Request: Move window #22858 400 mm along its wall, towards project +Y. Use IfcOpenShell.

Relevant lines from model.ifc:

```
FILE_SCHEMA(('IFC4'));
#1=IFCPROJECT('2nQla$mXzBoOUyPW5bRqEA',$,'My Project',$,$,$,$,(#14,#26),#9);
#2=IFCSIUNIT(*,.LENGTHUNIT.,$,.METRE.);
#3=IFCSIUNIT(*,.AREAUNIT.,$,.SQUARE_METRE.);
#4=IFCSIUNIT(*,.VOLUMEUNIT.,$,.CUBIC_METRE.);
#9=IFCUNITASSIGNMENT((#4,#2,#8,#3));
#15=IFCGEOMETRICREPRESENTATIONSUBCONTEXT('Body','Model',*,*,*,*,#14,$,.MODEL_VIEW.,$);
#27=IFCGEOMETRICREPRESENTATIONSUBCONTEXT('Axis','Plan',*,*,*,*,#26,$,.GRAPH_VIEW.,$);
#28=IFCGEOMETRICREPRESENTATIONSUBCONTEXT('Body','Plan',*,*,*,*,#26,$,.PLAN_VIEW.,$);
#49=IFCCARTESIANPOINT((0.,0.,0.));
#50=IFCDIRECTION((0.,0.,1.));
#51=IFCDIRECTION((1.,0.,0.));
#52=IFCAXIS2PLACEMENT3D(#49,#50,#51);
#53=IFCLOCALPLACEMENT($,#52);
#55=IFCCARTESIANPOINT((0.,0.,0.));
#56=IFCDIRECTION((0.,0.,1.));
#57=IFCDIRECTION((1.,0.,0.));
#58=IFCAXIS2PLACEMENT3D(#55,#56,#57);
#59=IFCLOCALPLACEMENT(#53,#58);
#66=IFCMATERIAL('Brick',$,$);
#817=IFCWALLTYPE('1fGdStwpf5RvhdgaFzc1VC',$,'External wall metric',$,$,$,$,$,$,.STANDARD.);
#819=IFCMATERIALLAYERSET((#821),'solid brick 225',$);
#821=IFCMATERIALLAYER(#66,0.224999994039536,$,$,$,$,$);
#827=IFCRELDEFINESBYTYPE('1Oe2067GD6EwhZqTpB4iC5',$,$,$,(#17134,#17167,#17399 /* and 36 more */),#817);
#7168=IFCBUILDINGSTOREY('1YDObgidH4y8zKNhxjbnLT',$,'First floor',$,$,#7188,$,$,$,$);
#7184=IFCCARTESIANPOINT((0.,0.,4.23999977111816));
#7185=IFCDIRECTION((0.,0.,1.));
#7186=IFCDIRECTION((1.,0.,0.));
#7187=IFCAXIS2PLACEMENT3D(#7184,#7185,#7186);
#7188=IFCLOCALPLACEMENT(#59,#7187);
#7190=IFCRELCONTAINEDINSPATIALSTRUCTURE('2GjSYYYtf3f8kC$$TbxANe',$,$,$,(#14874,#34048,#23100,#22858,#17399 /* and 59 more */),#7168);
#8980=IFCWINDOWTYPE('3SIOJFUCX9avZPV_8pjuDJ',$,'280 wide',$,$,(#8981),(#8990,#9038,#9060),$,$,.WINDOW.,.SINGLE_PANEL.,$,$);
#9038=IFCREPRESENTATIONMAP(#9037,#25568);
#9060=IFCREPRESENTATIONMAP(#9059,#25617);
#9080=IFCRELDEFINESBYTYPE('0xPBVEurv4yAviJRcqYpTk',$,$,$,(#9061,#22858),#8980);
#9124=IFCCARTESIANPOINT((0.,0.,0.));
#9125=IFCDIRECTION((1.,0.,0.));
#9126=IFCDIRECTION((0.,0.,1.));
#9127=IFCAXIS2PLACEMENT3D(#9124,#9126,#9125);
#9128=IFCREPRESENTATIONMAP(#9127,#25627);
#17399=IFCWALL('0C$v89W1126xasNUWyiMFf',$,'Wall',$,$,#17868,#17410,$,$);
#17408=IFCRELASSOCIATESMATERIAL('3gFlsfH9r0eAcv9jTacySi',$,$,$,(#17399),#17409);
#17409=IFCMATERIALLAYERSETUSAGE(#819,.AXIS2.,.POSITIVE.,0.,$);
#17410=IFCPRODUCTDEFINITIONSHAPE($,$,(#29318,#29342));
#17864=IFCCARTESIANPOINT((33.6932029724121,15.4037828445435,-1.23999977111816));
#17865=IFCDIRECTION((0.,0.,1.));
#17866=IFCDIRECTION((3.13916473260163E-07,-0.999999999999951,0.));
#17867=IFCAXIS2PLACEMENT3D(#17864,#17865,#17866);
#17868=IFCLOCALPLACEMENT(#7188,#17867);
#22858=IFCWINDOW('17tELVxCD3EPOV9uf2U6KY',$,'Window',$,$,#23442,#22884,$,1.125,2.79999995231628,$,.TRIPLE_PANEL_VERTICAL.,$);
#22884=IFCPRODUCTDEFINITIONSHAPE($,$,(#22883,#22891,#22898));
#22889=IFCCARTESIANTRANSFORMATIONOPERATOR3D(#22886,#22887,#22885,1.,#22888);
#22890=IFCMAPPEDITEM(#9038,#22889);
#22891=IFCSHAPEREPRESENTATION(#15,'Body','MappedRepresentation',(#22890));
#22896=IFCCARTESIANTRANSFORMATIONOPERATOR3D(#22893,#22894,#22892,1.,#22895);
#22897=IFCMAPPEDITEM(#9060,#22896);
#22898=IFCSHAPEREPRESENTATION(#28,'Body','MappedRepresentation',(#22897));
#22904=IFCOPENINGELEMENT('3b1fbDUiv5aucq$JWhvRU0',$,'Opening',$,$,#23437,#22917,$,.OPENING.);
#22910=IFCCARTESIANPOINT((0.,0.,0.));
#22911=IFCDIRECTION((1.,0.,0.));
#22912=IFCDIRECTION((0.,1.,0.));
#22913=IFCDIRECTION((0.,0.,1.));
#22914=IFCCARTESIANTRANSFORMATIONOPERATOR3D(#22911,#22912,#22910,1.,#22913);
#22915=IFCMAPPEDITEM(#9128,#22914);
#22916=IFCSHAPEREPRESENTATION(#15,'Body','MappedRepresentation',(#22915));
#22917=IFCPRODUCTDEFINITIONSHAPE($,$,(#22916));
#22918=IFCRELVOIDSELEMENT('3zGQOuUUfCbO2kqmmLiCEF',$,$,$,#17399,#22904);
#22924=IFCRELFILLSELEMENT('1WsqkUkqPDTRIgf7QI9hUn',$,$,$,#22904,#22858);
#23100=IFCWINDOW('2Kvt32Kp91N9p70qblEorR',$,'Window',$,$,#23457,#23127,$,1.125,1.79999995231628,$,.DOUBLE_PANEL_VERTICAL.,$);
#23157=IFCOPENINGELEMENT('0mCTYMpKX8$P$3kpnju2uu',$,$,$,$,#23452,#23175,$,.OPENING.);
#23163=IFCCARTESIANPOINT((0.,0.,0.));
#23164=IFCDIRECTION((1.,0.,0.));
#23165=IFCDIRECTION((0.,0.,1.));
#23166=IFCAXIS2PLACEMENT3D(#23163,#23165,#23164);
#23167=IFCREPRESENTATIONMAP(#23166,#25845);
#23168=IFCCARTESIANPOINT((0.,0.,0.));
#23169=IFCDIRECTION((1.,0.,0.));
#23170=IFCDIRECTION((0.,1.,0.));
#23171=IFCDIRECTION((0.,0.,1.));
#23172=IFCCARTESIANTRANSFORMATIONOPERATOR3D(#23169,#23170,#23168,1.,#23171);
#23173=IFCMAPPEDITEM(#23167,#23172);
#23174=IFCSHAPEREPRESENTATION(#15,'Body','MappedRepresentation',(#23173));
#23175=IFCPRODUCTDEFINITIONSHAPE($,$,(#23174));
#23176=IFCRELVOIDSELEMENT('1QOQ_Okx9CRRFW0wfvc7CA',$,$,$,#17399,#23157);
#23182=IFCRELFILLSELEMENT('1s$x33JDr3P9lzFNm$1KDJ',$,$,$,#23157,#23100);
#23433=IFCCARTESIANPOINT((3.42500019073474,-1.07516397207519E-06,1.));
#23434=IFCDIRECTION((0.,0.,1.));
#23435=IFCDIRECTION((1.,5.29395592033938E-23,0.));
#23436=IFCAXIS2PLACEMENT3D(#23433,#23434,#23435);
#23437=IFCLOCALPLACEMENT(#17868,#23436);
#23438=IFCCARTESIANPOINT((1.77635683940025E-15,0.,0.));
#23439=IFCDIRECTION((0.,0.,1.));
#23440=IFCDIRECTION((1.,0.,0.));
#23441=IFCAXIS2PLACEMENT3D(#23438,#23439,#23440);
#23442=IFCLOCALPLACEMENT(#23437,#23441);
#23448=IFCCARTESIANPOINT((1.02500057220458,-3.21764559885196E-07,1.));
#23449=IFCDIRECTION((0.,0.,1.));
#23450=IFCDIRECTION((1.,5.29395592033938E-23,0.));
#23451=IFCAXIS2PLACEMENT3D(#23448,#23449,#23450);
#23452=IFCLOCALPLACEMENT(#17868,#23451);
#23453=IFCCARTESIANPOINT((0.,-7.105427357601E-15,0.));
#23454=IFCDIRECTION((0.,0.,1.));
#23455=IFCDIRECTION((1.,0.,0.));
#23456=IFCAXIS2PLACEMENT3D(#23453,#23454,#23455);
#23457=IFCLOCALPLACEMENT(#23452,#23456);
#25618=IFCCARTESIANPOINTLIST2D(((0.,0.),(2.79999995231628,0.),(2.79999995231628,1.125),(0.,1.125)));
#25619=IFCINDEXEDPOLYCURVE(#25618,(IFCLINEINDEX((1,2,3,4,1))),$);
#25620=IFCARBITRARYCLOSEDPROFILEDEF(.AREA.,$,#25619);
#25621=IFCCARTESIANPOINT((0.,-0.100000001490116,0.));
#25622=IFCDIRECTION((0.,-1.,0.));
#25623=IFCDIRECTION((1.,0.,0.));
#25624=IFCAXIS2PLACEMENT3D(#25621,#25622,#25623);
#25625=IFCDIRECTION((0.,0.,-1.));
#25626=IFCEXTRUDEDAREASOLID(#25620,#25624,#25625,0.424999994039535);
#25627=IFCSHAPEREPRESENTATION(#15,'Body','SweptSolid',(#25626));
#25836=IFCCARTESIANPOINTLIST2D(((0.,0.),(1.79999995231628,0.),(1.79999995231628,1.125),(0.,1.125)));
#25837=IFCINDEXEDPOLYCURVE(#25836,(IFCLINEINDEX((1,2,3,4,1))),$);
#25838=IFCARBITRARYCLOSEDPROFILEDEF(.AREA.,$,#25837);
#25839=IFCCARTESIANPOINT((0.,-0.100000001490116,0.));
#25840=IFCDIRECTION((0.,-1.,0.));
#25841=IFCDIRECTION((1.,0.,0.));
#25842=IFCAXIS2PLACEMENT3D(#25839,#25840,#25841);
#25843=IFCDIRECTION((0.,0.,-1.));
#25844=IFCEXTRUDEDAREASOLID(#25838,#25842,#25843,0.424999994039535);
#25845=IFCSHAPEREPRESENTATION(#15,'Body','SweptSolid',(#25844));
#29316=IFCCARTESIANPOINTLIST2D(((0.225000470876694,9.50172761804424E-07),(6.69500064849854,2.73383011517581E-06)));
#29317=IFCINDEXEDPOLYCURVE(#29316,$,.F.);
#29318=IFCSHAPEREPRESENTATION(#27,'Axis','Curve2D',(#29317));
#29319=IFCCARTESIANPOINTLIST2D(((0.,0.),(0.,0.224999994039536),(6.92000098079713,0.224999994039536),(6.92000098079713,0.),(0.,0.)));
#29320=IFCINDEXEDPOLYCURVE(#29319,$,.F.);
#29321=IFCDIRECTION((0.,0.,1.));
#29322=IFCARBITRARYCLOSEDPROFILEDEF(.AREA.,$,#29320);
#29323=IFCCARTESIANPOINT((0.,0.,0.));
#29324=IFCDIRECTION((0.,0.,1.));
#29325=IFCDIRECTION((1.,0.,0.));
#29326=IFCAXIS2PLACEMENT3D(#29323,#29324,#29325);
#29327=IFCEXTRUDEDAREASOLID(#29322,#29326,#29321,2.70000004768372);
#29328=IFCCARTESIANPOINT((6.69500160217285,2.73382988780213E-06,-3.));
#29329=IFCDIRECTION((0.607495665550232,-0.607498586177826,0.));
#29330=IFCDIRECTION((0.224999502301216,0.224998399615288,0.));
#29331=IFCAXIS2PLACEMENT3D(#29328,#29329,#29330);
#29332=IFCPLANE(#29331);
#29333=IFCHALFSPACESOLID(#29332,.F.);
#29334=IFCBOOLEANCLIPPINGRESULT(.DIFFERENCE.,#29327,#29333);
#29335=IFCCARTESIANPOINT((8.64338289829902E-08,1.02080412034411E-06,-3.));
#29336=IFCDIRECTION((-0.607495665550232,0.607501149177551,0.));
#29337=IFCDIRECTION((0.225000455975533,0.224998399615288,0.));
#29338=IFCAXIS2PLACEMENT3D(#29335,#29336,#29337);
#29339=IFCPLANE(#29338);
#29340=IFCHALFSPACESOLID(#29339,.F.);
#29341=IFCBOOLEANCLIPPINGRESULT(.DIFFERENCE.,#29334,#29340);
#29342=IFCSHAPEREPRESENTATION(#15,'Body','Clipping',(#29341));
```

```python
import ifcopenshell
import ifcopenshell.api.geometry
import ifcopenshell.util.placement
import ifcopenshell.util.unit

model = ifcopenshell.open("model.ifc")
unit_scale = ifcopenshell.util.unit.calculate_unit_scale(model)

window = model.by_guid("17tELVxCD3EPOV9uf2U6KY")
opening = window.FillsVoids[0].RelatingOpeningElement
wall = opening.VoidsElements[0].RelatingBuildingElement

wall_matrix = ifcopenshell.util.placement.get_local_placement(wall.ObjectPlacement)
shift = wall_matrix[:3, 0] * -0.4 / unit_scale
before = ifcopenshell.util.placement.get_local_placement(window.ObjectPlacement)[:3, 3].copy()

# The window is placed relative to its opening, so it follows when the opening moves.
matrix = ifcopenshell.util.placement.get_local_placement(opening.ObjectPlacement)
matrix[:3, 3] += shift
ifcopenshell.api.geometry.edit_object_placement(
    model, product=opening, matrix=matrix, is_si=False, should_transform_children=True
)

after = ifcopenshell.util.placement.get_local_placement(window.ObjectPlacement)[:3, 3]
print("window moved by", (after - before).round(3) + 0.0)

model.write("model_updated.ifc")
```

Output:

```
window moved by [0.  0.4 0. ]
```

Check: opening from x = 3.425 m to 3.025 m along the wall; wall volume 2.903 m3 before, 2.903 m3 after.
